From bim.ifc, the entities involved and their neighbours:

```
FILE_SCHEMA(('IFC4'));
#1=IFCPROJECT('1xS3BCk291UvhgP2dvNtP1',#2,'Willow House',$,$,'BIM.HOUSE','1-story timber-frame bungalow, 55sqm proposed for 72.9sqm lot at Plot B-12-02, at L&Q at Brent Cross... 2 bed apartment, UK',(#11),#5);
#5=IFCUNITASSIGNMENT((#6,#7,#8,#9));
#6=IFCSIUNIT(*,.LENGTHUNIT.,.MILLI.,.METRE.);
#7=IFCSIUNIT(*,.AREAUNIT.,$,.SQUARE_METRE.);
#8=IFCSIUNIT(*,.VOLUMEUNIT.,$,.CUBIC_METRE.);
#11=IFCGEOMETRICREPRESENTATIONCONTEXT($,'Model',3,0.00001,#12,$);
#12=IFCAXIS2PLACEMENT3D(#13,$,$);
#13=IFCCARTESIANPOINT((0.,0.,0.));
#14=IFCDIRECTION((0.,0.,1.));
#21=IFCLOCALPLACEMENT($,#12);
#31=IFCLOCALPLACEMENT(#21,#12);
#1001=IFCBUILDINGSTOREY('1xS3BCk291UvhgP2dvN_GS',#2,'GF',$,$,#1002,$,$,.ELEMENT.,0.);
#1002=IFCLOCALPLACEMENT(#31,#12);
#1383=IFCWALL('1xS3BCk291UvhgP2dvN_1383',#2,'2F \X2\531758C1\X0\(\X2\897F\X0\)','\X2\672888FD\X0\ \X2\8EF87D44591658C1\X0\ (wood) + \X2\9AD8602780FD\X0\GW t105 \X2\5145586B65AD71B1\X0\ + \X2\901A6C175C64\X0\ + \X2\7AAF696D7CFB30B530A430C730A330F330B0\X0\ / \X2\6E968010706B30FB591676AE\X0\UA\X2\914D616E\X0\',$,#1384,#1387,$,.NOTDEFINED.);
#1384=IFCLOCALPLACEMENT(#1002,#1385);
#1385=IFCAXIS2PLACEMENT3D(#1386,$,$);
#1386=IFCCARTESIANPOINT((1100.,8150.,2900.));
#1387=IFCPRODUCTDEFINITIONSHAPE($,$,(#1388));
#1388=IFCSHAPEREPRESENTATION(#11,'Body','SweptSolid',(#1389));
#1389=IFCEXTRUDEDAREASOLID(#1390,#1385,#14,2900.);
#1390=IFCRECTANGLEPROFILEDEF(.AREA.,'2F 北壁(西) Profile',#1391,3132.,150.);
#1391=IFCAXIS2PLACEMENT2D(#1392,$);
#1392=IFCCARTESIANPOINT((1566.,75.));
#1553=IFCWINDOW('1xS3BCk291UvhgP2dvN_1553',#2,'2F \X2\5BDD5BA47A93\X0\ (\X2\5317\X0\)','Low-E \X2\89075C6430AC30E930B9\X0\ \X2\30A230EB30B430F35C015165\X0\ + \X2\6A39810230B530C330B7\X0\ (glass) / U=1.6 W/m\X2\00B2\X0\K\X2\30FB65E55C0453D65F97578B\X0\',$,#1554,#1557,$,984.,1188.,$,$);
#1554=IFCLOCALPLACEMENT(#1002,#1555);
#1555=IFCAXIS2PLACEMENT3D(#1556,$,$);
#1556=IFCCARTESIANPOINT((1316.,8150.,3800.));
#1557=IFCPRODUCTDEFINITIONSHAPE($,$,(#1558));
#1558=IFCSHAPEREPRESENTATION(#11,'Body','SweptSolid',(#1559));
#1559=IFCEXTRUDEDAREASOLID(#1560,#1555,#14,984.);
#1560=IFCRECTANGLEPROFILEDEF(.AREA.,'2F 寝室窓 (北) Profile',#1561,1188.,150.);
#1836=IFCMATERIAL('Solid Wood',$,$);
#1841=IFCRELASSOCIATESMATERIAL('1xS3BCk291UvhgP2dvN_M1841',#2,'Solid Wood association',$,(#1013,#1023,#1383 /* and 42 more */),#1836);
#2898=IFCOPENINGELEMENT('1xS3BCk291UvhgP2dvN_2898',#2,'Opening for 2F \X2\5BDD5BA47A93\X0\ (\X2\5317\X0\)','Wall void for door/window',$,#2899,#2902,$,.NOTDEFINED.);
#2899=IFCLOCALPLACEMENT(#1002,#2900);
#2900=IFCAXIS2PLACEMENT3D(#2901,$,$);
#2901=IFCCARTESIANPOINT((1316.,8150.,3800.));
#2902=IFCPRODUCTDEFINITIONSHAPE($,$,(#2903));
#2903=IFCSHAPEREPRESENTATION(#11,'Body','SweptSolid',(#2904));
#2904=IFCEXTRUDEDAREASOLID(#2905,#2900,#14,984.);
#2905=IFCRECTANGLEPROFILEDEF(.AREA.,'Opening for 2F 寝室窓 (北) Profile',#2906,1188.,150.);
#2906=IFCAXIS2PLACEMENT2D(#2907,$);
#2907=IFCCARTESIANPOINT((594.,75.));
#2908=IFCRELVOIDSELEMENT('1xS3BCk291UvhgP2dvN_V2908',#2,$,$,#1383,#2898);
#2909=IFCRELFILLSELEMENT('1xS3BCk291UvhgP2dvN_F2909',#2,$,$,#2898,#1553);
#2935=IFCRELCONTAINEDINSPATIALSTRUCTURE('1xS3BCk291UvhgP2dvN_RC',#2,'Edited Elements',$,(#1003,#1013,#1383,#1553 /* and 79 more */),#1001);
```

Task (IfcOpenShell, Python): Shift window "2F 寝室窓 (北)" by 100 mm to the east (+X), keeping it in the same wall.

```python
import ifcopenshell
import ifcopenshell.api.geometry
import ifcopenshell.util.placement

model = ifcopenshell.open("bim.ifc")

window = model.by_id(1553)
opening = window.FillsVoids[0].RelatingOpeningElement
wall = opening.VoidsElements[0].RelatingBuildingElement

wall_matrix = ifcopenshell.util.placement.get_local_placement(wall.ObjectPlacement)
shift = wall_matrix[:3, 0] * 100.0
before = ifcopenshell.util.placement.get_local_placement(window.ObjectPlacement)[:3, 3].copy()

# The window is not placed relative to its opening, so move both.
for product in (opening, window):
    matrix = ifcopenshell.util.placement.get_local_placement(product.ObjectPlacement)
    matrix[:3, 3] += shift
    ifcopenshell.api.geometry.edit_object_placement(model, product=product, matrix=matrix, is_si=False)

after = ifcopenshell.util.placement.get_local_placement(window.ObjectPlacement)[:3, 3]
print("window moved by", (after - before).round(3) + 0.0)

model.write("bim_v2.ifc")
```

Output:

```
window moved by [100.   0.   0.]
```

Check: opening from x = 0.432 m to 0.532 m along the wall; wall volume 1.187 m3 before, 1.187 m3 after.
